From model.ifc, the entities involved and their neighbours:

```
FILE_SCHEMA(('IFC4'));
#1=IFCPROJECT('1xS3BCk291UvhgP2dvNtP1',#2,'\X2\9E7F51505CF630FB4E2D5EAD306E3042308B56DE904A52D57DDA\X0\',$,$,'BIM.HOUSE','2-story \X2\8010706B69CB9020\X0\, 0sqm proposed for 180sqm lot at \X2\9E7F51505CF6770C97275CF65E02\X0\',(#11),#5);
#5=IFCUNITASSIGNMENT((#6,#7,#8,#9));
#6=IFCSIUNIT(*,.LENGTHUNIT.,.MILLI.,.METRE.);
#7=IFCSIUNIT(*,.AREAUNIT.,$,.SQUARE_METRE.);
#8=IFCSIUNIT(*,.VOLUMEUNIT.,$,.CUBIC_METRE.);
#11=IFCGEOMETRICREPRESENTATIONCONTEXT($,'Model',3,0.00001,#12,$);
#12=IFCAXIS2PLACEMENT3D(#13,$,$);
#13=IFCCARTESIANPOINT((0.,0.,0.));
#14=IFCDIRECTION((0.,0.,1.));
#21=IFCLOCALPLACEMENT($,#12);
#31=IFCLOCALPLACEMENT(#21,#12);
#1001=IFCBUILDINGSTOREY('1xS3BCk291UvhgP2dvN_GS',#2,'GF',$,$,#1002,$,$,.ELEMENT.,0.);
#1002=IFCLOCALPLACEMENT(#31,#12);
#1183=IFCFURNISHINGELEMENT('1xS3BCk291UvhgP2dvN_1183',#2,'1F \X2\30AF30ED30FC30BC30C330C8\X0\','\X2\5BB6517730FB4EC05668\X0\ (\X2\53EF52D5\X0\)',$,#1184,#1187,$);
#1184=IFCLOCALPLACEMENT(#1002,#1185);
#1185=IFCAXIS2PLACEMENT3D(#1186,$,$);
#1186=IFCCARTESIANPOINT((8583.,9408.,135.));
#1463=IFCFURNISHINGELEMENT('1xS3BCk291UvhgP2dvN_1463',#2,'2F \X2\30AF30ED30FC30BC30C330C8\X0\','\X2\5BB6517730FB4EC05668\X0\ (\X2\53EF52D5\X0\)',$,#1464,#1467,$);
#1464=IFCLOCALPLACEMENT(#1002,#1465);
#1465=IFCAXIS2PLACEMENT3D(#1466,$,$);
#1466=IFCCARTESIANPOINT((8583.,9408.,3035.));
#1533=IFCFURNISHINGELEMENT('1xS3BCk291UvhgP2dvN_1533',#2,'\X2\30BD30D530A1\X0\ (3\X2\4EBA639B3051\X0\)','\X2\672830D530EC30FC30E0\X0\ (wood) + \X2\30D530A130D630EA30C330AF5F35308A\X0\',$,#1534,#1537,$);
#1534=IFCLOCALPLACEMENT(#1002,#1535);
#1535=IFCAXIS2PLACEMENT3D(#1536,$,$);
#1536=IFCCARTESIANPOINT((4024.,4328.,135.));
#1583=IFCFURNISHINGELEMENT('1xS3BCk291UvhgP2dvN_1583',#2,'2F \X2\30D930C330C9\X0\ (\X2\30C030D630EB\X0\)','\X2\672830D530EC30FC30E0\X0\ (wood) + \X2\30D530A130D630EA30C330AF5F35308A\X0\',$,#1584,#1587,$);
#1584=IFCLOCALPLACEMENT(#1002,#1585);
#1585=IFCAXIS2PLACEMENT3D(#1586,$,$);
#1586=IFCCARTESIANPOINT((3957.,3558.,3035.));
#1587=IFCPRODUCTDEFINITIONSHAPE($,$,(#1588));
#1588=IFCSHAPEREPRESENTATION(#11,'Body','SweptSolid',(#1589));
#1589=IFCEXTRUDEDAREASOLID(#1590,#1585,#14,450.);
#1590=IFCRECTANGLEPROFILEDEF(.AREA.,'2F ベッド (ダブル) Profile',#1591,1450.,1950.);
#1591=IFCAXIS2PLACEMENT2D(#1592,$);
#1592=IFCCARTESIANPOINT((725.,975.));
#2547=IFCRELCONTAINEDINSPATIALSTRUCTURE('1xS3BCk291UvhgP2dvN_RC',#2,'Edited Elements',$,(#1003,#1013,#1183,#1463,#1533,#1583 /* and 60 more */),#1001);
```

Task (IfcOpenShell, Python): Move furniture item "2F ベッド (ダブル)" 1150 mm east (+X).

```python
import ifcopenshell
import ifcopenshell.api.geometry
import ifcopenshell.util.placement
import ifcopenshell.util.unit

model = ifcopenshell.open("model.ifc")
unit_scale = ifcopenshell.util.unit.calculate_unit_scale(model)

item = model.by_id(1583)
matrix = ifcopenshell.util.placement.get_local_placement(item.ObjectPlacement)
matrix[0, 3] += 1.15 / unit_scale
ifcopenshell.api.geometry.edit_object_placement(model, product=item, matrix=matrix, is_si=False)

print(ifcopenshell.util.placement.get_local_placement(item.ObjectPlacement).round(3) + 0.0)

model.write("model-out.ifc")
```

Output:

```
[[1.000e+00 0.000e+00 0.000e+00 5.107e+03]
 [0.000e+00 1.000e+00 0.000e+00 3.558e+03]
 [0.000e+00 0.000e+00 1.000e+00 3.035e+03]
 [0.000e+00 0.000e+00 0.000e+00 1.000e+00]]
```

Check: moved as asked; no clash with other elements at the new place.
